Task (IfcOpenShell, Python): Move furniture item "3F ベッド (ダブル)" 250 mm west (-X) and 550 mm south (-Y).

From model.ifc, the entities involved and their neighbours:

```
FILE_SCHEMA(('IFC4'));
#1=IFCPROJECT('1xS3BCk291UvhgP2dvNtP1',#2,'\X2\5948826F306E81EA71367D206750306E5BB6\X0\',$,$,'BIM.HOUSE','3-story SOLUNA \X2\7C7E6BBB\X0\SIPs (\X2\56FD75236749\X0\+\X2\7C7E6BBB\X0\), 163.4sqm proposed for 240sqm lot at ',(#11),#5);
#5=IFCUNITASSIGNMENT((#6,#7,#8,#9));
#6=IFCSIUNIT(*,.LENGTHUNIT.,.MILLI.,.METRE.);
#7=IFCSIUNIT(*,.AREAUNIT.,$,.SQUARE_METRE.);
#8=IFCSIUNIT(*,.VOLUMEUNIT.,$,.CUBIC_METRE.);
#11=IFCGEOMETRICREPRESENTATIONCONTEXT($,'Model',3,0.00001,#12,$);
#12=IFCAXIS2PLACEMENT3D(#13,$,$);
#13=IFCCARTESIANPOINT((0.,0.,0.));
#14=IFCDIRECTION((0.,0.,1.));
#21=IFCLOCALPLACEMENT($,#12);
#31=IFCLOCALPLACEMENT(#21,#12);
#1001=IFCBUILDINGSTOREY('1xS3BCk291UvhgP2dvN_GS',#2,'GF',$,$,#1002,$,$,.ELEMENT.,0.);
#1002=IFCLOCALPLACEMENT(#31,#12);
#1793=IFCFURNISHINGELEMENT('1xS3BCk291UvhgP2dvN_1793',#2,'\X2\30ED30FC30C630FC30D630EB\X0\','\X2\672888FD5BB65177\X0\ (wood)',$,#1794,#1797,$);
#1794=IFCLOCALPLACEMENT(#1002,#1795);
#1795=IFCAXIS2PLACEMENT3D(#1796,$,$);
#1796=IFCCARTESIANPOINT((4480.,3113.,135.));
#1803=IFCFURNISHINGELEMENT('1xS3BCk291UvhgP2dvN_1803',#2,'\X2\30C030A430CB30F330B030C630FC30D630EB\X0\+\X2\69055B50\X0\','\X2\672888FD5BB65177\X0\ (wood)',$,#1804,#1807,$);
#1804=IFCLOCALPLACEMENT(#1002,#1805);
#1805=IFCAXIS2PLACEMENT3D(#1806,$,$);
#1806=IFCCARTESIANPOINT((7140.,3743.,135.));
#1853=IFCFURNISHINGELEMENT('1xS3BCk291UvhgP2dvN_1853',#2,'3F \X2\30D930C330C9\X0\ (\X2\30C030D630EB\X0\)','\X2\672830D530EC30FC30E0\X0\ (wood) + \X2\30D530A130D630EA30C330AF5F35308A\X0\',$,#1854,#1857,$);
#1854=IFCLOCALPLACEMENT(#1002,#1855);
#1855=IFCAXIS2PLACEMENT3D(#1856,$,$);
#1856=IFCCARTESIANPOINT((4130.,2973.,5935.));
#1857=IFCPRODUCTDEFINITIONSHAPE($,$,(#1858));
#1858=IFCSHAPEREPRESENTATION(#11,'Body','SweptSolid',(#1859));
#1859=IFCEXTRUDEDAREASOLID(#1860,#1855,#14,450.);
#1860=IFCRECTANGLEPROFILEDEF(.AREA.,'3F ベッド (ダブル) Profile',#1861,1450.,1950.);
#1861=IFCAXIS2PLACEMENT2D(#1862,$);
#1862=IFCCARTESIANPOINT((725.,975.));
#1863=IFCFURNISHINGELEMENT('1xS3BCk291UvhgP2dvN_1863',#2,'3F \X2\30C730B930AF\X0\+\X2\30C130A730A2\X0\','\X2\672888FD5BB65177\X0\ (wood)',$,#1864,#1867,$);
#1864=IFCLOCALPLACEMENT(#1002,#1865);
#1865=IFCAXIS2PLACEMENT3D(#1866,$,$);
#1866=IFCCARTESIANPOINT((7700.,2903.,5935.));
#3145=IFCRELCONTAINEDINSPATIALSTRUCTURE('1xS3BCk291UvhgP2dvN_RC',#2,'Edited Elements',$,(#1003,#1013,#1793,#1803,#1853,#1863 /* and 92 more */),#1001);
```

```python
import ifcopenshell
import ifcopenshell.api.geometry
import ifcopenshell.util.placement
import ifcopenshell.util.unit

model = ifcopenshell.open("model.ifc")
unit_scale = ifcopenshell.util.unit.calculate_unit_scale(model)

item = model.by_id(1853)
matrix = ifcopenshell.util.placement.get_local_placement(item.ObjectPlacement)
matrix[0, 3] -= 0.25 / unit_scale
matrix[1, 3] -= 0.55 / unit_scale
ifcopenshell.api.geometry.edit_object_placement(model, product=item, matrix=matrix, is_si=False)

print(ifcopenshell.util.placement.get_local_placement(item.ObjectPlacement).round(3) + 0.0)

model.write("model_rev.ifc")
```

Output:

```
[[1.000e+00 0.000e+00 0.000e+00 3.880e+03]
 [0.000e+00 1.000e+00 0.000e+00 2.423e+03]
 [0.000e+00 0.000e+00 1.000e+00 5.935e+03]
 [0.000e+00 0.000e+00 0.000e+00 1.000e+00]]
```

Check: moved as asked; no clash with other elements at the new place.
